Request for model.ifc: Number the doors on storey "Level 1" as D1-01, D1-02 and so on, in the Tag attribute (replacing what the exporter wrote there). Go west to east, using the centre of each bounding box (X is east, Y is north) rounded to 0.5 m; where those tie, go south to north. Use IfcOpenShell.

First a look at what the model holds.

```python
import ifcopenshell
import ifcopenshell.util.element
import ifcopenshell.util.placement

model = ifcopenshell.open("model.ifc")
print(model.schema)
storey = next(s for s in model.by_type("IfcBuildingStorey") if s.Name == "Level 1")
doors = [e for e in ifcopenshell.util.element.get_decomposition(storey) if e.is_a("IfcDoor")]
for e in sorted(doors, key=lambda e: e.id()):
    origin = ifcopenshell.util.placement.get_local_placement(e.ObjectPlacement)[:3, 3]
    print(e.id(), e.Tag, e.Name, origin.round(2) + 0.0, sep=" | ")
```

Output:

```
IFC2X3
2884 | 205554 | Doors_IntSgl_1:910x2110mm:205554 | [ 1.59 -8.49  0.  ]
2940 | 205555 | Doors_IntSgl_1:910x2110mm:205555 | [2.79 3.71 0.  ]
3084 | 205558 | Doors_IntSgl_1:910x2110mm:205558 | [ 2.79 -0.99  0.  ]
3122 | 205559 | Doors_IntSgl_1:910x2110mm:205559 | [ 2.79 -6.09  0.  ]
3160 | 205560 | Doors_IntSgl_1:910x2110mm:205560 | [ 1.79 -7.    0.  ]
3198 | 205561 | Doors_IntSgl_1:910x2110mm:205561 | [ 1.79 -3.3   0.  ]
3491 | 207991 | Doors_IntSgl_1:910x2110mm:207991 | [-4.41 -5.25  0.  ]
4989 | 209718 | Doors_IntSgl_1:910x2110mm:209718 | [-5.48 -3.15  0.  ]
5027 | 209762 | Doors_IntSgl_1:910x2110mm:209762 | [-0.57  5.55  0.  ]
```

```python
import ifcopenshell
import ifcopenshell.geom
import ifcopenshell.util.element
import ifcopenshell.util.shape

model = ifcopenshell.open("model.ifc")
settings = ifcopenshell.geom.settings()
settings.set("use-world-coords", True)


def centre(element):
    shape = ifcopenshell.geom.create_shape(settings, element)
    return ifcopenshell.util.shape.get_bbox_centroid(shape.geometry)


storey = next(s for s in model.by_type("IfcBuildingStorey") if s.Name == "Level 1")
doors = [e for e in ifcopenshell.util.element.get_decomposition(storey) if e.is_a("IfcDoor")]

# Insertion points can sit at a corner or the storey origin, so sort by the geometry (in metres).
centres = {e: centre(e) for e in doors}
doors.sort(key=lambda e: (round(centres[e][0] / 0.5), centres[e][1]))

for i, e in enumerate(doors, start=1):
    number = f"D1-{i:02d}"
    e.Tag = number
    print(e.id(), number)

model.write("model_v2.ifc")
```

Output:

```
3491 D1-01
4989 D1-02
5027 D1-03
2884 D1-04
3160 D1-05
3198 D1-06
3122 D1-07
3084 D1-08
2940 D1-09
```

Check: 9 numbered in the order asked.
